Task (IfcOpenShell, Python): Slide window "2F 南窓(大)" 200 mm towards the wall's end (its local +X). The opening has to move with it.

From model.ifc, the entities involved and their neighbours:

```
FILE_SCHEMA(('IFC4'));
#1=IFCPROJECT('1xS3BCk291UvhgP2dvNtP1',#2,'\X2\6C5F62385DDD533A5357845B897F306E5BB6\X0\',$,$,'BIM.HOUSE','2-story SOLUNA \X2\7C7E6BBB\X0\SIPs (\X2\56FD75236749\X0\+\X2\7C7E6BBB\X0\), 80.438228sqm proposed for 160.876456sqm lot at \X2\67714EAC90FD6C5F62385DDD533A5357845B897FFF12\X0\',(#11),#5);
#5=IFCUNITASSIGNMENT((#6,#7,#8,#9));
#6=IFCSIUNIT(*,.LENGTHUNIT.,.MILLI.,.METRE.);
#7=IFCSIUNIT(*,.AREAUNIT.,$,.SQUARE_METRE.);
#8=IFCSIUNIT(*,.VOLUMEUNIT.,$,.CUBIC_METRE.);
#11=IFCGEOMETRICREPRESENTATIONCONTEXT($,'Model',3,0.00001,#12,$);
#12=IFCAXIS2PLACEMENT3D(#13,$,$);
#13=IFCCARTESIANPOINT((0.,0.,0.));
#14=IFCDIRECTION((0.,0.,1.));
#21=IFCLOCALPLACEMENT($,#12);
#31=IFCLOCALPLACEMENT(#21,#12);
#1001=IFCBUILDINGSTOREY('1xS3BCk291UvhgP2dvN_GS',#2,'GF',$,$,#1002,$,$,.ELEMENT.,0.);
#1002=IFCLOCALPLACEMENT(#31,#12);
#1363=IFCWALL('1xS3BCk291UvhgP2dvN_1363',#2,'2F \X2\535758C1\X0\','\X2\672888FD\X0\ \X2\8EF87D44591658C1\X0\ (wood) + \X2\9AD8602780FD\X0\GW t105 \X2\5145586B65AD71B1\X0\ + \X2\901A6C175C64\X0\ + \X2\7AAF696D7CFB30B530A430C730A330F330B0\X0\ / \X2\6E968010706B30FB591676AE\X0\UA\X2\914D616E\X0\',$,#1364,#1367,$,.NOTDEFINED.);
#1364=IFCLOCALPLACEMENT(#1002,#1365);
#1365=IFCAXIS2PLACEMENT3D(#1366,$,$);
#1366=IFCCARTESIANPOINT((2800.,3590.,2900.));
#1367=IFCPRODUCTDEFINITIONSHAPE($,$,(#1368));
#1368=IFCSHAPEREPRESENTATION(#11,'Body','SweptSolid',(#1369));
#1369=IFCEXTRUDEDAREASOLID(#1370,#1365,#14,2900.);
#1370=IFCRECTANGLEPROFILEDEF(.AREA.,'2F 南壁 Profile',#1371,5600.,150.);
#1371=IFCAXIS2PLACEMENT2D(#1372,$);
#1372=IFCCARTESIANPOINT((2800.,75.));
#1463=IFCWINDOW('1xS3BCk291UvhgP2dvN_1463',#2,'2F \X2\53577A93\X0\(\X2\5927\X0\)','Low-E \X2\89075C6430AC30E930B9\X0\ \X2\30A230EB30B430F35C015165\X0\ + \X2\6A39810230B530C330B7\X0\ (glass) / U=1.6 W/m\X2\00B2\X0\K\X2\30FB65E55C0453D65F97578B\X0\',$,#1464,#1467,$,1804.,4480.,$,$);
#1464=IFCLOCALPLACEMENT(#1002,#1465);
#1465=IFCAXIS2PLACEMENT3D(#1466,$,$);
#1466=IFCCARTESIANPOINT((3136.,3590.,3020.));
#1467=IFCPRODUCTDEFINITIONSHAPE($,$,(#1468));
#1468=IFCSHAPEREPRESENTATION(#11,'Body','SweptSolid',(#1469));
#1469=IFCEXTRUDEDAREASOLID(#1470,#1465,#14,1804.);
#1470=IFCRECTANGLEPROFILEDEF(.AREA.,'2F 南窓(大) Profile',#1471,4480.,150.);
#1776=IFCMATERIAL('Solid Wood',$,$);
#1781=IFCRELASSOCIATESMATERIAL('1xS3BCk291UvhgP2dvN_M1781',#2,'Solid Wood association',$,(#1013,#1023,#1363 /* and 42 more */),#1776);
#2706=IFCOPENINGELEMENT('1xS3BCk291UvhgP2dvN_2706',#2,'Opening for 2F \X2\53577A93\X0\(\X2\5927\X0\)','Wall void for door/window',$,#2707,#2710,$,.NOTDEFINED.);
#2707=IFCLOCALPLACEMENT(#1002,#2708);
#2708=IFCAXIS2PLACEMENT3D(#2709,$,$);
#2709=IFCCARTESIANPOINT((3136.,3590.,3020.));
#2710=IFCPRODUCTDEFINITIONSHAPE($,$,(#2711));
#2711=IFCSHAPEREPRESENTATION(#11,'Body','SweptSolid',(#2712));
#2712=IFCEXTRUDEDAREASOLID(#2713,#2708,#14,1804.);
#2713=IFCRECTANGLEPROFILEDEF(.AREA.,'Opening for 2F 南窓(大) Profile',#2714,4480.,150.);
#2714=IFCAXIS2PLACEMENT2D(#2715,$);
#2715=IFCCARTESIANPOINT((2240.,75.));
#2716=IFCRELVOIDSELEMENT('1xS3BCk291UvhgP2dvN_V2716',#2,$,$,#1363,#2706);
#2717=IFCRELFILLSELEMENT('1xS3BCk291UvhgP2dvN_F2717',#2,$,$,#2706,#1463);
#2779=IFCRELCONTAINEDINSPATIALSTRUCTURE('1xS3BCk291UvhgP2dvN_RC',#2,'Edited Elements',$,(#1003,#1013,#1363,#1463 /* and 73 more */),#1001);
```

```python
import ifcopenshell
import ifcopenshell.api.geometry
import ifcopenshell.util.placement
import ifcopenshell.util.unit

model = ifcopenshell.open("model.ifc")
unit_scale = ifcopenshell.util.unit.calculate_unit_scale(model)

window = model.by_guid("1xS3BCk291UvhgP2dvN_1463")
opening = window.FillsVoids[0].RelatingOpeningElement
wall = opening.VoidsElements[0].RelatingBuildingElement

wall_matrix = ifcopenshell.util.placement.get_local_placement(wall.ObjectPlacement)
shift = wall_matrix[:3, 0] * 0.2 / unit_scale
before = ifcopenshell.util.placement.get_local_placement(window.ObjectPlacement)[:3, 3].copy()

# The window is not placed relative to its opening, so move both.
for product in (opening, window):
    matrix = ifcopenshell.util.placement.get_local_placement(product.ObjectPlacement)
    matrix[:3, 3] += shift
    ifcopenshell.api.geometry.edit_object_placement(model, product=product, matrix=matrix, is_si=False)

after = ifcopenshell.util.placement.get_local_placement(window.ObjectPlacement)[:3, 3]
print("window moved by", (after - before).round(3) + 0.0)

model.write("model_v2.ifc")
```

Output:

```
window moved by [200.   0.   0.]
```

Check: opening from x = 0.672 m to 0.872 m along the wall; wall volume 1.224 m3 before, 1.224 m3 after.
